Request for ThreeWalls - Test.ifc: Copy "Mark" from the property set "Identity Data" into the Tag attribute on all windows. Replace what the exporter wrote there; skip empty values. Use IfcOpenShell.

First a look at what the model holds.

```python
import ifcopenshell
import ifcopenshell.util.element

model = ifcopenshell.open("ThreeWalls - Test.ifc")
print(model.schema)
windows = model.by_type("IfcWindow")
print(len(windows), "windows")
for e in windows[:8]:
    source = ifcopenshell.util.element.get_pset(e, "Identity Data", "Mark")
    target = e.Tag
    print(e.id(), repr(source), repr(target), sep=" | ")
```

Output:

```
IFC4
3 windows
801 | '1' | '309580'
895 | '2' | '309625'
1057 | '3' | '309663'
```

```python
import ifcopenshell
import ifcopenshell.util.element

model = ifcopenshell.open("ThreeWalls - Test.ifc")

count = 0
for e in model.by_type("IfcWindow"):
    value = ifcopenshell.util.element.get_pset(e, "Identity Data", "Mark")
    current = e.Tag
    if not value or not value.strip() or current == value:
        continue
    e.Tag = value
    count += 1

print(count, "windows updated")

model.write("ThreeWalls - Test_updated.ifc")
```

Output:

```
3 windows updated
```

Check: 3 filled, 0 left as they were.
